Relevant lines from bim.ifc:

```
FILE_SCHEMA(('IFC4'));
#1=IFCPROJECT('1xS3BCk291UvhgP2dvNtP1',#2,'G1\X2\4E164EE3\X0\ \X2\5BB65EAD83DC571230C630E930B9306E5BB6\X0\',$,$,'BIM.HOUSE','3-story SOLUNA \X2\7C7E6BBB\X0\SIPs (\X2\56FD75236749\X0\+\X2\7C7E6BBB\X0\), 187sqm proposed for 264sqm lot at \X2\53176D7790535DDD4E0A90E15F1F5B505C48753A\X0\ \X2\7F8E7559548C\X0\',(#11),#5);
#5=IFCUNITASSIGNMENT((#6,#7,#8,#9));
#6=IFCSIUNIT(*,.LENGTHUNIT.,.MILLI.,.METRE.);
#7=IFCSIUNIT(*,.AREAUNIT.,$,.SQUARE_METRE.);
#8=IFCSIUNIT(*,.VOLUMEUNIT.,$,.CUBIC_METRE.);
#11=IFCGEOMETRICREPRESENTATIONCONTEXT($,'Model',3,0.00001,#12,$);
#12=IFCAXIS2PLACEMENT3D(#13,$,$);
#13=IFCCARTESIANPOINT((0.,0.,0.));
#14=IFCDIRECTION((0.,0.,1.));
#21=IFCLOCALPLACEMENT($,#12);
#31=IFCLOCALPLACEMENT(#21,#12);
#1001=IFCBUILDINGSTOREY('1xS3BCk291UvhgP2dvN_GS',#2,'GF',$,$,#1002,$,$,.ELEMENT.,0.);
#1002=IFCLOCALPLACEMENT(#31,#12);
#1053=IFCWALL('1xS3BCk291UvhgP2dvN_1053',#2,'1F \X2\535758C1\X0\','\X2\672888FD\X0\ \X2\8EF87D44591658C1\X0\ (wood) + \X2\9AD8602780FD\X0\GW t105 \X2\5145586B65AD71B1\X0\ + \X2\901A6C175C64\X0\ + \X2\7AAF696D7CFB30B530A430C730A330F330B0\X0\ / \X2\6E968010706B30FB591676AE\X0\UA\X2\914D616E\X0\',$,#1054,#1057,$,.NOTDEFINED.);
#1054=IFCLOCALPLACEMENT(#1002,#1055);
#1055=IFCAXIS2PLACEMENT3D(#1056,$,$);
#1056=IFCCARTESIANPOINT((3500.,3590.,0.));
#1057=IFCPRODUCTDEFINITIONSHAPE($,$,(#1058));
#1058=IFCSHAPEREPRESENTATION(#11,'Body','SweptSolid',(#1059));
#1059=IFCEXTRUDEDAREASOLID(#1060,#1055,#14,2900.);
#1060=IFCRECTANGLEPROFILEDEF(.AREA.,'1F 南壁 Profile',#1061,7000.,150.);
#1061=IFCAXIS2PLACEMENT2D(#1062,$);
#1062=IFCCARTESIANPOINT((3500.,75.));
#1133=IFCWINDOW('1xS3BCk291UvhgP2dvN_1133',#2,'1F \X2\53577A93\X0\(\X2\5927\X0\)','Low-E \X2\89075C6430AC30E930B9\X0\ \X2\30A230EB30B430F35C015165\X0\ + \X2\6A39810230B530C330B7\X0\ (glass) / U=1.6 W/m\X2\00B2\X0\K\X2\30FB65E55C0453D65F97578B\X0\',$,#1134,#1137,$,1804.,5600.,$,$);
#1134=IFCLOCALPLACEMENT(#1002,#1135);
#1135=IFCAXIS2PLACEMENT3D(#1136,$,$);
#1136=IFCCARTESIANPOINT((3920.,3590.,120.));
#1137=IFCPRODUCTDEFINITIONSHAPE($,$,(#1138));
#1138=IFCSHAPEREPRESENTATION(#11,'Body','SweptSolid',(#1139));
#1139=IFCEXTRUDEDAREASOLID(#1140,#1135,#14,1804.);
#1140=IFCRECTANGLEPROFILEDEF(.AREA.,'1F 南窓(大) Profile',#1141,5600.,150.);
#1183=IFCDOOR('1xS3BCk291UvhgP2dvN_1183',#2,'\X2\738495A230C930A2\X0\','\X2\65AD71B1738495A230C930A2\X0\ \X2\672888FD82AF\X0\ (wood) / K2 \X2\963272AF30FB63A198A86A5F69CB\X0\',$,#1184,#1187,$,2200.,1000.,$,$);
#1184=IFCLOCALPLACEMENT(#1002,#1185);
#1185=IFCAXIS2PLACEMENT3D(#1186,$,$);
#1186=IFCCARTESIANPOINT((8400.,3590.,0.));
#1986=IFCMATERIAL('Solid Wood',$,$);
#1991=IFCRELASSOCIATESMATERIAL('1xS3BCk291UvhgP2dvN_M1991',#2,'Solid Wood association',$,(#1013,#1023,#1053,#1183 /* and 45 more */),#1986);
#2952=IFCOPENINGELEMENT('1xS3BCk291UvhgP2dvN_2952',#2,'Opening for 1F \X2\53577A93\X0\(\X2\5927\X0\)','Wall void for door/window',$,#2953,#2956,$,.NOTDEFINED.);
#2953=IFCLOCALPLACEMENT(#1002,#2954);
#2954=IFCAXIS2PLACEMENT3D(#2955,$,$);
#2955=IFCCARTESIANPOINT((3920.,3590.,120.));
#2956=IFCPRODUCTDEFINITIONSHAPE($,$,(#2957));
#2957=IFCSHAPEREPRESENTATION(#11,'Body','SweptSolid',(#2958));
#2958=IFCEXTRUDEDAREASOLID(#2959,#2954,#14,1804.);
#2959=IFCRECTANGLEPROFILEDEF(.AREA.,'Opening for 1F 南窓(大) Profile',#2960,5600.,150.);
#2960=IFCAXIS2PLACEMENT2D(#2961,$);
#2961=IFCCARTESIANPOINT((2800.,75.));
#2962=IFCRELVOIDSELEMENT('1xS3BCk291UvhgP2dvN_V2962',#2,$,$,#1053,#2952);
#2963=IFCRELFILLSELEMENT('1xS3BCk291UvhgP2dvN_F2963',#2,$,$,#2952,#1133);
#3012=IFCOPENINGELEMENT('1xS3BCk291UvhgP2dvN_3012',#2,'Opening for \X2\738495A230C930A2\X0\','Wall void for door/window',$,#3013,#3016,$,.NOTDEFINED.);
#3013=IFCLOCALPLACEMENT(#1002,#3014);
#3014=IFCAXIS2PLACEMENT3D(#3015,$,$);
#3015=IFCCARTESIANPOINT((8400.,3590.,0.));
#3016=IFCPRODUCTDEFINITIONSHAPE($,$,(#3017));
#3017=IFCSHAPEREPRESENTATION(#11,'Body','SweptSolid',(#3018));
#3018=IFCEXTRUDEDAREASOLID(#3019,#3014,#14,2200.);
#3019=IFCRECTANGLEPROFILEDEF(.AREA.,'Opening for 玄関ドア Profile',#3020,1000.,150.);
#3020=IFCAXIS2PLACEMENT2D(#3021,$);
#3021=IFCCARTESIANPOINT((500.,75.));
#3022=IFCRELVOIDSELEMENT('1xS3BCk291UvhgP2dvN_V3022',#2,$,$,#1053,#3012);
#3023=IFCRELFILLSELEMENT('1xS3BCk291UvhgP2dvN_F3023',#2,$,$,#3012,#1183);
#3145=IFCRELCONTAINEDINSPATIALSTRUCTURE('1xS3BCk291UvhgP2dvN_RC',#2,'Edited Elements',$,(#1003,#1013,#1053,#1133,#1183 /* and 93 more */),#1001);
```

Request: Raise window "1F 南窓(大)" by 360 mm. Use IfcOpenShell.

```python
import numpy as np
import ifcopenshell
import ifcopenshell.api.geometry
import ifcopenshell.util.placement
import ifcopenshell.util.unit

model = ifcopenshell.open("bim.ifc")
unit_scale = ifcopenshell.util.unit.calculate_unit_scale(model)

window = model.by_guid("1xS3BCk291UvhgP2dvN_1133")
opening = window.FillsVoids[0].RelatingOpeningElement
dz = 0.36 / unit_scale

shift = np.array([0.0, 0.0, dz])
# The window is not placed relative to its opening, so move both.
for product in (opening, window):
    matrix = ifcopenshell.util.placement.get_local_placement(product.ObjectPlacement)
    matrix[:3, 3] += shift
    ifcopenshell.api.geometry.edit_object_placement(model, product=product, matrix=matrix, is_si=False)

print(f"moved by {dz * unit_scale:+.3f} m")

model.write("bim-out.ifc")
```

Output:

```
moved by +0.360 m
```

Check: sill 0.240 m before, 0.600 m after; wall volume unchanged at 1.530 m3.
